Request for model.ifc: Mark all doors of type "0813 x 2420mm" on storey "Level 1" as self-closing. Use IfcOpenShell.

First a look at what the model holds.

```python
import ifcopenshell
import ifcopenshell.util.element

model = ifcopenshell.open("model.ifc")
print(model.schema)
storey = next(s for s in model.by_type("IfcBuildingStorey") if s.Name == "Level 1")
doors = [e for e in ifcopenshell.util.element.get_decomposition(storey) if e.is_a("IfcDoor")]
seen = {}
for e in doors:
    element_type = ifcopenshell.util.element.get_type(e)
    key = (element_type.Name if element_type != e and element_type else None, ifcopenshell.util.element.get_pset(e, "Pset_DoorCommon", "SelfClosing"))
    seen[key] = seen.get(key, 0) + 1
for (name, value), count in sorted(seen.items(), key=str):
    print(count, "x", name, "|", value)
```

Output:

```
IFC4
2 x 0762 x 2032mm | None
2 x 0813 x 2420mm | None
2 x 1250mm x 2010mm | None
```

```python
import ifcopenshell
import ifcopenshell.api.pset
import ifcopenshell.util.element

model = ifcopenshell.open("model.ifc")

storey = next(s for s in model.by_type("IfcBuildingStorey") if s.Name == "Level 1")
doors = [e for e in ifcopenshell.util.element.get_decomposition(storey) if e.is_a("IfcDoor")]

count = 0
for e in doors:
    element_type = ifcopenshell.util.element.get_type(e)
    if element_type in (None, e) or element_type.Name != "0813 x 2420mm":
        continue
    # add_pset returns the element's existing set when there is one.
    pset = ifcopenshell.api.pset.add_pset(model, product=e, name="Pset_DoorCommon")
    ifcopenshell.api.pset.edit_pset(model, pset=pset, properties={"SelfClosing": True})
    count += 1

print(count, "doors updated")

model.write("model_rev.ifc")
```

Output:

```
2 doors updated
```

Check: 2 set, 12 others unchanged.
